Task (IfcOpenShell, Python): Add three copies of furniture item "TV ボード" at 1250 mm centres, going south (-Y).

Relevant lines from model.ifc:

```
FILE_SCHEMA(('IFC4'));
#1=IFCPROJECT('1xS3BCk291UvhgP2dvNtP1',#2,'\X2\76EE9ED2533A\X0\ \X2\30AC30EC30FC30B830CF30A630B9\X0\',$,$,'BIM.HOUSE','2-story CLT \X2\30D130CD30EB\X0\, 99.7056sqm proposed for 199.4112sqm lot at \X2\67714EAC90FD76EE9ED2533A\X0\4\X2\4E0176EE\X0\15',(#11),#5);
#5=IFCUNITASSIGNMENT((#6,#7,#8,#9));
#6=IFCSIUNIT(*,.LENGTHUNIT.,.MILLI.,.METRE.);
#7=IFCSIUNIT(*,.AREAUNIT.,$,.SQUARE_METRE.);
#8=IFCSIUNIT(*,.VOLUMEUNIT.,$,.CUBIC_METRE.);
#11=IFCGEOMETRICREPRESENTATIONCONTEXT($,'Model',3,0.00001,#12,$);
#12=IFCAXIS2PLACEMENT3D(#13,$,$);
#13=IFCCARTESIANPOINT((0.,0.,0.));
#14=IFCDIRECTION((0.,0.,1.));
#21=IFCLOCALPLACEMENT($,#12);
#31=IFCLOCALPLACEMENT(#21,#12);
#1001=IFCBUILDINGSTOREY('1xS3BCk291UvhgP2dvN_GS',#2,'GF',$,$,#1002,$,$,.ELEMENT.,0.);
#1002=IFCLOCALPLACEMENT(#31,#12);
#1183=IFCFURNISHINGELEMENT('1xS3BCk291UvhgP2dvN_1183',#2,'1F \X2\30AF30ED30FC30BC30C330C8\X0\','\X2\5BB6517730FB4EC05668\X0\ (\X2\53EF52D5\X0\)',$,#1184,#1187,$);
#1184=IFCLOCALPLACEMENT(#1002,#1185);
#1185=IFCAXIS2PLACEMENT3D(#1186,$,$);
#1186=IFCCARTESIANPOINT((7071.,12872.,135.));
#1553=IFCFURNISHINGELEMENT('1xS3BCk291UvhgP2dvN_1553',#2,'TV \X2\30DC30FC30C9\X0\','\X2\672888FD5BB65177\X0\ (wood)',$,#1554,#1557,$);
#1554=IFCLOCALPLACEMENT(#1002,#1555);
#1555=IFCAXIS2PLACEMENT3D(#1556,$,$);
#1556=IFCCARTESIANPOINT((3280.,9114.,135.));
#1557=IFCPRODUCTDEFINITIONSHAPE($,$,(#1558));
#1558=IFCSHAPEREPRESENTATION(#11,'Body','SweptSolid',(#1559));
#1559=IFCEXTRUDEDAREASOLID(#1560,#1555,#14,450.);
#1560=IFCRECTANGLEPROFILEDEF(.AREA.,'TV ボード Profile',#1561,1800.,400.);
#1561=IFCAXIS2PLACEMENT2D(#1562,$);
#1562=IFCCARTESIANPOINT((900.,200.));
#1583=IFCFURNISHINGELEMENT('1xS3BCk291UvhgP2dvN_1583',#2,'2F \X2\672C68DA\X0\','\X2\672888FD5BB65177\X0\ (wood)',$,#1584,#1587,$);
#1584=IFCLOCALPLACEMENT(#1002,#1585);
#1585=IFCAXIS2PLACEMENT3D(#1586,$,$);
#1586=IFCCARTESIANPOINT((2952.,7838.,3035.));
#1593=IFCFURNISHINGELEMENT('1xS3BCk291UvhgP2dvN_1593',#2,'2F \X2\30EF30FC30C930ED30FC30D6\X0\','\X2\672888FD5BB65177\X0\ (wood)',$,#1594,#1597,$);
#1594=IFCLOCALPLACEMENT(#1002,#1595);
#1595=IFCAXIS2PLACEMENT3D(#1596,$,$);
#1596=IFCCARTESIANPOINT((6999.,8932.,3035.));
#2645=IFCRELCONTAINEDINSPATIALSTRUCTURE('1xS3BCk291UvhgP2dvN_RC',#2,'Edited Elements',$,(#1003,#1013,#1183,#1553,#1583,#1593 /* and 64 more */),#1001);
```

```python
import numpy as np
import ifcopenshell
import ifcopenshell.api.geometry
import ifcopenshell.api.root
import ifcopenshell.util.element
import ifcopenshell.util.placement

model = ifcopenshell.open("model.ifc")


def reuse_history(source, copy):
    """copy_class also copies each property set's owner history, people and application; keep the originals."""
    for rel in copy.IsDefinedBy:
        if rel.is_a("IfcRelDefinesByProperties") and (history := rel.RelatingPropertyDefinition.OwnerHistory):
            rel.RelatingPropertyDefinition.OwnerHistory = source.OwnerHistory
            ifcopenshell.util.element.remove_deep2(model, history)


source = model.by_guid("1xS3BCk291UvhgP2dvN_1553")
base = ifcopenshell.util.placement.get_local_placement(source.ObjectPlacement)
step = np.array([0.0, -1.0, 0.0]) * 1250.0

for i in range(1, 4):
    copy = ifcopenshell.api.root.copy_class(model, product=source)
    copy.Representation = ifcopenshell.util.element.copy_deep(
        model, source.Representation, exclude=["IfcGeometricRepresentationContext", "IfcRepresentationMap"]
    )
    reuse_history(source, copy)
    matrix = base.copy()
    matrix[:3, 3] += i * step
    print("added at", matrix[:3, 3].round(3) + 0.0)
    ifcopenshell.api.geometry.edit_object_placement(model, product=copy, matrix=matrix, is_si=False)

model.write("model_rev.ifc")
```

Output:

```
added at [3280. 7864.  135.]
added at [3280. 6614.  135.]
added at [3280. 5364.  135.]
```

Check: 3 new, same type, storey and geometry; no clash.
